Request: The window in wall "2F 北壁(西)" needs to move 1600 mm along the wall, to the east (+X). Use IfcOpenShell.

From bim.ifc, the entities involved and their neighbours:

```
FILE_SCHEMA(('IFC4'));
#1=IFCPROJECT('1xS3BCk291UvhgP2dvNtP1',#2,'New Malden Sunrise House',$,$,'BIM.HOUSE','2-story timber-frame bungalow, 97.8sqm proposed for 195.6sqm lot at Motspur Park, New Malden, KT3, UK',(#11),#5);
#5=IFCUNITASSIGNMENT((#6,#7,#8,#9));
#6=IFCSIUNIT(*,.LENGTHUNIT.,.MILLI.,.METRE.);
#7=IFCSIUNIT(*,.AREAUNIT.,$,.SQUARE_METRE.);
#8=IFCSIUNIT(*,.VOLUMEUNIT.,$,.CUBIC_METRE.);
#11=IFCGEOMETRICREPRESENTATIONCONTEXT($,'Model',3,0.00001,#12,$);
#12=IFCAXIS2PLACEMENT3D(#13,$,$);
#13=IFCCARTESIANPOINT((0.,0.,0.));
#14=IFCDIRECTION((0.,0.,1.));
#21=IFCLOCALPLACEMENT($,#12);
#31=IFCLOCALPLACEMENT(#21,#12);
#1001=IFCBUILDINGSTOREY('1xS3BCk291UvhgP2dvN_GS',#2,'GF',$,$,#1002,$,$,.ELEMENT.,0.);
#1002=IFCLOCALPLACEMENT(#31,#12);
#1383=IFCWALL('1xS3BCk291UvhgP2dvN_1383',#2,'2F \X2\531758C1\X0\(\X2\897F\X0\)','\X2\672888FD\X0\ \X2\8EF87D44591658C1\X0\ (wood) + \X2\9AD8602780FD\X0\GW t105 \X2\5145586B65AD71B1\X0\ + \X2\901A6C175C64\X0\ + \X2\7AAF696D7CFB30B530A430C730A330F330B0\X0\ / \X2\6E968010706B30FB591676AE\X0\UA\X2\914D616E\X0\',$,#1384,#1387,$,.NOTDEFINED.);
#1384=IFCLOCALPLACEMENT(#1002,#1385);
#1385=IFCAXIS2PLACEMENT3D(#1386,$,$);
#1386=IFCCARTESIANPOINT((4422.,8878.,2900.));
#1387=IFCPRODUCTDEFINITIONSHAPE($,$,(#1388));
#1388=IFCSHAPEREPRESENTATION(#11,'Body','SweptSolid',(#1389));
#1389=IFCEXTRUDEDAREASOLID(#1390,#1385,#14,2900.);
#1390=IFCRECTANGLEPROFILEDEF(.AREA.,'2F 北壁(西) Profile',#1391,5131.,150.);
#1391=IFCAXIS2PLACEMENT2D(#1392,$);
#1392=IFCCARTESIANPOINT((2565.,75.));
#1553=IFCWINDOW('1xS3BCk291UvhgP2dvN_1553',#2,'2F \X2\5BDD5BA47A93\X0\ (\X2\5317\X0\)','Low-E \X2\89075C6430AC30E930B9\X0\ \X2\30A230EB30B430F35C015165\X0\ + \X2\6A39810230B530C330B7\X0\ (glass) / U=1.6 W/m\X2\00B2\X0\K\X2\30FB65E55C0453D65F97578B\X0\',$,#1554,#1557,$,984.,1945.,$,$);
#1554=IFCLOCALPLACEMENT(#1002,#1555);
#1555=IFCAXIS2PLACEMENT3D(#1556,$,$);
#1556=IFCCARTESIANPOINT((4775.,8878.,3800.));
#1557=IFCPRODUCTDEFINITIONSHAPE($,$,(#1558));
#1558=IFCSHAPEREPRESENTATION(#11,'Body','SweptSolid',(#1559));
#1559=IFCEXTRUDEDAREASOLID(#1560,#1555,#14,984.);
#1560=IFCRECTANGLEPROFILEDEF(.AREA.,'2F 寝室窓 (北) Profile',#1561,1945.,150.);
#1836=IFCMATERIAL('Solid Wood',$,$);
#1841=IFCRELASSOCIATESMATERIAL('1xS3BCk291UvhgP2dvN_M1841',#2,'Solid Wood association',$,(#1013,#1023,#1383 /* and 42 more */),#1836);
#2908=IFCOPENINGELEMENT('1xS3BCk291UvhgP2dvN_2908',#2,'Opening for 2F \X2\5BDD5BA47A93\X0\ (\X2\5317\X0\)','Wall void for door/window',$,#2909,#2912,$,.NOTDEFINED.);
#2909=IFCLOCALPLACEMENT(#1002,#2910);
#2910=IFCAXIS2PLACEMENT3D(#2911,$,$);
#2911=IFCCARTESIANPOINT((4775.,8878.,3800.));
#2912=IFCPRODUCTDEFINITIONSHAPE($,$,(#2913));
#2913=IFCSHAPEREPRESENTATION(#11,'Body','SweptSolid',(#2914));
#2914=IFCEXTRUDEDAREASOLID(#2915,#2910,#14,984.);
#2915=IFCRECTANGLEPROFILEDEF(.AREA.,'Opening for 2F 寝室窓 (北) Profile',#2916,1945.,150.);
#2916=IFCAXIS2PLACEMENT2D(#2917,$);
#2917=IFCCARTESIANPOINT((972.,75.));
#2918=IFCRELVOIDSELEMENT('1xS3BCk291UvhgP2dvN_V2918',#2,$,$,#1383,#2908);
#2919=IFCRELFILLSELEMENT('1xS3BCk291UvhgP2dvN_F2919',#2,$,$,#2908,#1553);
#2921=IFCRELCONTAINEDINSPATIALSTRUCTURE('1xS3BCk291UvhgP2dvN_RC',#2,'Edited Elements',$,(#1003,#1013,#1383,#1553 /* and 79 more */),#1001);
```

```python
import ifcopenshell
import ifcopenshell.api.geometry
import ifcopenshell.util.placement

model = ifcopenshell.open("bim.ifc")

window = model.by_guid("1xS3BCk291UvhgP2dvN_1553")
opening = window.FillsVoids[0].RelatingOpeningElement
wall = opening.VoidsElements[0].RelatingBuildingElement

wall_matrix = ifcopenshell.util.placement.get_local_placement(wall.ObjectPlacement)
shift = wall_matrix[:3, 0] * 1600.0
before = ifcopenshell.util.placement.get_local_placement(window.ObjectPlacement)[:3, 3].copy()

# The window is not placed relative to its opening, so move both.
for product in (opening, window):
    matrix = ifcopenshell.util.placement.get_local_placement(product.ObjectPlacement)
    matrix[:3, 3] += shift
    ifcopenshell.api.geometry.edit_object_placement(model, product=product, matrix=matrix, is_si=False)

after = ifcopenshell.util.placement.get_local_placement(window.ObjectPlacement)[:3, 3]
print("window moved by", (after - before).round(3) + 0.0)

model.write("bim_rev.ifc")
```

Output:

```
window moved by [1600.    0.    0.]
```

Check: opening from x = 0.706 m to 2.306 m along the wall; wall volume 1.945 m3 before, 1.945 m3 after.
